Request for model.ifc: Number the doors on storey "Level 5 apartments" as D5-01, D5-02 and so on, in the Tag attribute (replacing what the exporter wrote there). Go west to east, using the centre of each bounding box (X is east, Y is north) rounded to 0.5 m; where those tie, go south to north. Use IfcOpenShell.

First a look at what the model holds.

```python
import ifcopenshell
import ifcopenshell.util.element
import ifcopenshell.util.placement

model = ifcopenshell.open("model.ifc")
print(model.schema)
storey = next(s for s in model.by_type("IfcBuildingStorey") if s.Name == "Level 5 apartments")
doors = [e for e in ifcopenshell.util.element.get_decomposition(storey) if e.is_a("IfcDoor")]
for e in sorted(doors, key=lambda e: e.id()):
    origin = ifcopenshell.util.placement.get_local_placement(e.ObjectPlacement)[:3, 3]
    print(e.id(), e.Tag, e.Name, origin.round(2) + 0.0, sep=" | ")
```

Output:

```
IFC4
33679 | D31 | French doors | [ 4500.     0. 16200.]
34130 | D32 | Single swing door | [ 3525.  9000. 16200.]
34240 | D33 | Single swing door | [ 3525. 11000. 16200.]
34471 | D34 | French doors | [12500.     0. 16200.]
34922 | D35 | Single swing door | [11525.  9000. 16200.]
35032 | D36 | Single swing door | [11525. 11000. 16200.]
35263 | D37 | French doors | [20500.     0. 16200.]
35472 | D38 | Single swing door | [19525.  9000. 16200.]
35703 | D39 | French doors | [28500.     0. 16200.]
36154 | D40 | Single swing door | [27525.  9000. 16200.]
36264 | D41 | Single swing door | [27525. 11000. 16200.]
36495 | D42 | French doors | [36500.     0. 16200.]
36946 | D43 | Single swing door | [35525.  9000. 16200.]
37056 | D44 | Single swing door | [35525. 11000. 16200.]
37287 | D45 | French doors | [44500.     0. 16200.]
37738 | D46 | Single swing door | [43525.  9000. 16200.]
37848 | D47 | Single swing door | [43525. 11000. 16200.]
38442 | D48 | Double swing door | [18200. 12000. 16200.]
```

```python
import ifcopenshell
import ifcopenshell.geom
import ifcopenshell.util.element
import ifcopenshell.util.shape

model = ifcopenshell.open("model.ifc")
settings = ifcopenshell.geom.settings()
settings.set("use-world-coords", True)


def centre(element):
    shape = ifcopenshell.geom.create_shape(settings, element)
    return ifcopenshell.util.shape.get_bbox_centroid(shape.geometry)


storey = next(s for s in model.by_type("IfcBuildingStorey") if s.Name == "Level 5 apartments")
doors = [e for e in ifcopenshell.util.element.get_decomposition(storey) if e.is_a("IfcDoor")]

# Insertion points can sit at a corner or the storey origin, so sort by the geometry (in metres).
centres = {e: centre(e) for e in doors}
doors.sort(key=lambda e: (round(centres[e][0] / 0.5), centres[e][1]))

for i, e in enumerate(doors, start=1):
    number = f"D5-{i:02d}"
    e.Tag = number
    print(e.id(), number)

model.write("model-out.ifc")
```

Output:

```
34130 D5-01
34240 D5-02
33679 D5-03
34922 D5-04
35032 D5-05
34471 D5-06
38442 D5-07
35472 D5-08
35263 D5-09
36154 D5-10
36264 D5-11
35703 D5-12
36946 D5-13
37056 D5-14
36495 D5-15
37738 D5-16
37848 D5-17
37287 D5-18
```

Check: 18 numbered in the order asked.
